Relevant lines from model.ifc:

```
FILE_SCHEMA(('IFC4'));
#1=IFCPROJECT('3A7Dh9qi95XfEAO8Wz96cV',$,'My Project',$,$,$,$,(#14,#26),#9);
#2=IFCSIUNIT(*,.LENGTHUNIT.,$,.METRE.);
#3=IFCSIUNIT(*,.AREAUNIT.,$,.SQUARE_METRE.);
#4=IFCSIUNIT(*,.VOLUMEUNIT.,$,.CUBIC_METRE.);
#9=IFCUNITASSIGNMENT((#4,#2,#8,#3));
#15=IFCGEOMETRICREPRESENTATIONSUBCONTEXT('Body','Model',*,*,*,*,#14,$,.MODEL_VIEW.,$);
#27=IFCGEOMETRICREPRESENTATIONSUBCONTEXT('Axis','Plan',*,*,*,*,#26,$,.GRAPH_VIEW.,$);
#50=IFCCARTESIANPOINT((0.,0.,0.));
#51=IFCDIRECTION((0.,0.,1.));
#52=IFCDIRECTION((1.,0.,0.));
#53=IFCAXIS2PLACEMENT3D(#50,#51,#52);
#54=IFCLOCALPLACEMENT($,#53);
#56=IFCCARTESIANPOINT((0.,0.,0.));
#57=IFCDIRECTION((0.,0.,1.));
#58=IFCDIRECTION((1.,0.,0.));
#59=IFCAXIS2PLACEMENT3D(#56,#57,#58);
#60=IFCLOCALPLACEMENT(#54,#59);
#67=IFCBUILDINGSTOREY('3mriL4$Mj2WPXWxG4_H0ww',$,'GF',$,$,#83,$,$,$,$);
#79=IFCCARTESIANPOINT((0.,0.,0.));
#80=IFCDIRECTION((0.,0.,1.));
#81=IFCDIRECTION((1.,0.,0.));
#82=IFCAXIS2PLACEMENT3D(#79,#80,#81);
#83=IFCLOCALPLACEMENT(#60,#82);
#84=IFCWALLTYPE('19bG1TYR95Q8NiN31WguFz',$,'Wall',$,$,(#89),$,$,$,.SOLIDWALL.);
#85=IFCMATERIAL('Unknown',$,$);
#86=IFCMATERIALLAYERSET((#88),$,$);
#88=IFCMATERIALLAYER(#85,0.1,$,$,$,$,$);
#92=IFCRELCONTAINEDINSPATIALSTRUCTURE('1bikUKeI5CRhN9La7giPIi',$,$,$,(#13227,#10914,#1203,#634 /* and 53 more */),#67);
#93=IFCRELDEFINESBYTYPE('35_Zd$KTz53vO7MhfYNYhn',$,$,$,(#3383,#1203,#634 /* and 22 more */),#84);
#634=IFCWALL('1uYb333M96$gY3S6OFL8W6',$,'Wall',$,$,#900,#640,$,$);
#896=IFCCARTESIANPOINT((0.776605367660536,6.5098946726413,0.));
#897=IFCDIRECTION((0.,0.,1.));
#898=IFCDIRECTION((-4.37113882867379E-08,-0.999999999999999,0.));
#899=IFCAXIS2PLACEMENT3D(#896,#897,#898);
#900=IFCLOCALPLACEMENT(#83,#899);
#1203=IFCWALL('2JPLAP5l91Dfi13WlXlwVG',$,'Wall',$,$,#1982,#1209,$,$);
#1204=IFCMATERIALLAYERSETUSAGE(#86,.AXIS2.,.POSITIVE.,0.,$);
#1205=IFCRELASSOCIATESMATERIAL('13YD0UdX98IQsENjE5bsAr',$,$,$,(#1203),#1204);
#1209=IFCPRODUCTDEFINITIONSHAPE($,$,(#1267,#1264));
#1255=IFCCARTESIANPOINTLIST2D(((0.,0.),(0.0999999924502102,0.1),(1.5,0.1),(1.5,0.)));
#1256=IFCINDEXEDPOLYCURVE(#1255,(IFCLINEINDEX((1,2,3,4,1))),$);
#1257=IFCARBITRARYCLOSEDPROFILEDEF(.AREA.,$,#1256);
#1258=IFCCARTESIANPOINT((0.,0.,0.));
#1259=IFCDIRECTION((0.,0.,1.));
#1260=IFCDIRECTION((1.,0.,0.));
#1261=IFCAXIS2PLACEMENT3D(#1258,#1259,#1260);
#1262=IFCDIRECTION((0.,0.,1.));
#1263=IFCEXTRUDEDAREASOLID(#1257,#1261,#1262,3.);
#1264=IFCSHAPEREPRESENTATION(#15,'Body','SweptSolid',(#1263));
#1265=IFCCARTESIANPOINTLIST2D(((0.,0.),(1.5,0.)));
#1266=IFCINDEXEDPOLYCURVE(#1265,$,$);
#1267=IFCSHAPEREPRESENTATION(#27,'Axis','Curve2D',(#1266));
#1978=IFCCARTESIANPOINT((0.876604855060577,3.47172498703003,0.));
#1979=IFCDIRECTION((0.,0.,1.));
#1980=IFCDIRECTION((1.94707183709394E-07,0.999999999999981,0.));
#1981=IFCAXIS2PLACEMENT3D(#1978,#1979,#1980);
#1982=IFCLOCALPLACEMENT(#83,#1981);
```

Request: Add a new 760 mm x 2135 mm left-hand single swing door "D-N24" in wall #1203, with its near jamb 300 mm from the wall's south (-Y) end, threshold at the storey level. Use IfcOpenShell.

```python
import numpy as np
import ifcopenshell
import ifcopenshell.api.feature
import ifcopenshell.api.geometry
import ifcopenshell.api.root
import ifcopenshell.api.spatial
import ifcopenshell.geom
import ifcopenshell.util.element
import ifcopenshell.util.placement
import ifcopenshell.util.representation
import ifcopenshell.util.shape
import ifcopenshell.util.unit

model = ifcopenshell.open("model.ifc")
unit_scale = ifcopenshell.util.unit.calculate_unit_scale(model)
settings = ifcopenshell.geom.settings()


def volume(element):
    """Net volume in cubic metres, openings subtracted."""
    shape = ifcopenshell.geom.create_shape(settings, element)
    return ifcopenshell.util.shape.get_volume(shape.geometry)


wall = model.by_guid("2JPLAP5l91Dfi13WlXlwVG")
storey = ifcopenshell.util.element.get_container(wall, ifc_class="IfcBuildingStorey")
context = ifcopenshell.util.representation.get_context(model, "Model", "Body", "MODEL_VIEW")
before = volume(wall)

width, height, from_end, sill = 0.76, 2.135, 0.3, 0.0  # metres

# The wall runs along its own X axis, and the end named is its -X end.
wall_shape = ifcopenshell.geom.create_shape(settings, wall)
x, y, z = ifcopenshell.util.shape.get_vertices(wall_shape.geometry).T
start = x.min() + from_end
face, thickness = float(y.min()), float(y.max() - y.min())
wall_matrix = ifcopenshell.util.placement.get_local_placement(wall.ObjectPlacement)
level = ifcopenshell.util.placement.get_local_placement(storey.ObjectPlacement)[2, 3]


def in_wall(x, y):
    """Placement at x, y metres in the wall's axes, at sill height."""
    matrix = wall_matrix.copy()
    matrix[:, 3] = wall_matrix @ np.array([x / unit_scale, y / unit_scale, 0.0, 1.0])
    matrix[2, 3] = level + sill / unit_scale
    return matrix


# Opening: a box that overshoots both wall faces by 50 mm.
opening = ifcopenshell.api.root.create_entity(model, ifc_class="IfcOpeningElement", predefined_type="OPENING")
box = ifcopenshell.api.geometry.add_wall_representation(
    model, context=context, length=width, height=height, thickness=thickness + 0.1
)
ifcopenshell.api.geometry.assign_representation(model, product=opening, representation=box)
ifcopenshell.api.geometry.edit_object_placement(model, product=opening, matrix=in_wall(start, face - 0.05), is_si=False)
ifcopenshell.api.feature.add_feature(model, feature=opening, element=wall)

door = ifcopenshell.api.root.create_entity(model, ifc_class="IfcDoor", name="D-N24", predefined_type="DOOR")
door.OverallWidth, door.OverallHeight = width / unit_scale, height / unit_scale
door.OperationType = "SINGLE_SWING_LEFT"
body = ifcopenshell.api.geometry.add_door_representation(
    model,
    context=context,
    overall_width=door.OverallWidth,
    overall_height=door.OverallHeight,
    operation_type="SINGLE_SWING_LEFT",
    lining_properties={"LiningDepth": thickness / unit_scale, "ThresholdDepth": thickness / unit_scale},
)
ifcopenshell.api.geometry.assign_representation(model, product=door, representation=body)
ifcopenshell.api.spatial.assign_container(model, products=[door], relating_structure=storey)
ifcopenshell.api.feature.add_filling(model, opening=opening, element=door)

# The lining spans the wall, so the door starts at the wall face.
ifcopenshell.api.geometry.edit_object_placement(model, product=door, matrix=in_wall(start, face), is_si=False)

after = volume(wall)

print(f"wall volume {before:.3f} -> {after:.3f} m3")

model.write("model-out.ifc")
```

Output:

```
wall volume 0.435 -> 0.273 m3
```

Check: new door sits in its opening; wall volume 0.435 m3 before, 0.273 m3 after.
